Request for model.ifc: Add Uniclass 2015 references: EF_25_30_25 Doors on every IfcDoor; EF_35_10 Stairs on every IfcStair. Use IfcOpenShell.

First a look at what the model holds.

```python
import ifcopenshell

model = ifcopenshell.open("model.ifc")
print(model.schema)
print("classifications:", [c.Name for c in model.by_type("IfcClassification")])
for ifc_class in ("IfcDoor", "IfcRoof", "IfcStair", "IfcWall", "IfcWindow"):
    print(ifc_class, len(model.by_type(ifc_class)))
```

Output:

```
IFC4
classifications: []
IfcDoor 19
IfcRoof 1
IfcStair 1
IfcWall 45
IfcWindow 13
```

```python
import ifcopenshell
import ifcopenshell.api.classification

model = ifcopenshell.open("model.ifc")

system = ifcopenshell.api.classification.add_classification(model, classification="Uniclass 2015")

codes = {
    "IfcDoor": ("EF_25_30_25", "Doors"),
    "IfcStair": ("EF_35_10", "Stairs"),
}
for ifc_class, (code, name) in codes.items():
    products = model.by_type(ifc_class)
    ifcopenshell.api.classification.add_reference(
        model, products=products, classification=system, identification=code, name=name
    )
    print(code, len(products))

model.write("model_v2.ifc")
```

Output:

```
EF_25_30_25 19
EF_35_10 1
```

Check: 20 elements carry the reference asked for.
